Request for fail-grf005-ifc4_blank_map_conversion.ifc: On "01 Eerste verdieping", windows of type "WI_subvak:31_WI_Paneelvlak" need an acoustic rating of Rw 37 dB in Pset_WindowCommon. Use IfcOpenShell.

First a look at what the model holds.

```python
import ifcopenshell
import ifcopenshell.util.element

model = ifcopenshell.open("fail-grf005-ifc4_blank_map_conversion.ifc")
print(model.schema)
storey = next(s for s in model.by_type("IfcBuildingStorey") if s.Name == "01 Eerste verdieping")
windows = [e for e in ifcopenshell.util.element.get_decomposition(storey) if e.is_a("IfcWindow")]
seen = {}
for e in windows:
    element_type = ifcopenshell.util.element.get_type(e)
    key = (element_type.Name if element_type != e and element_type else None, ifcopenshell.util.element.get_pset(e, "Pset_WindowCommon", "AcousticRating"))
    seen[key] = seen.get(key, 0) + 1
for (name, value), count in sorted(seen.items(), key=str):
    print(count, "x", name, "|", value)
```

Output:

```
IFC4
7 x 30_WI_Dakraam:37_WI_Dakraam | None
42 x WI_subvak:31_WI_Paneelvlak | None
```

```python
import ifcopenshell
import ifcopenshell.api.pset
import ifcopenshell.util.element

model = ifcopenshell.open("fail-grf005-ifc4_blank_map_conversion.ifc")

storey = next(s for s in model.by_type("IfcBuildingStorey") if s.Name == "01 Eerste verdieping")
windows = [e for e in ifcopenshell.util.element.get_decomposition(storey) if e.is_a("IfcWindow")]

count = 0
for e in windows:
    element_type = ifcopenshell.util.element.get_type(e)
    if element_type in (None, e) or element_type.Name != "WI_subvak:31_WI_Paneelvlak":
        continue
    # add_pset returns the element's existing set when there is one.
    pset = ifcopenshell.api.pset.add_pset(model, product=e, name="Pset_WindowCommon")
    ifcopenshell.api.pset.edit_pset(model, pset=pset, properties={"AcousticRating": "Rw 37 dB"})
    count += 1

print(count, "windows updated")

model.write("fail-grf005-ifc4_blank_map_conversion-out.ifc")
```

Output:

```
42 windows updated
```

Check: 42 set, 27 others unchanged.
